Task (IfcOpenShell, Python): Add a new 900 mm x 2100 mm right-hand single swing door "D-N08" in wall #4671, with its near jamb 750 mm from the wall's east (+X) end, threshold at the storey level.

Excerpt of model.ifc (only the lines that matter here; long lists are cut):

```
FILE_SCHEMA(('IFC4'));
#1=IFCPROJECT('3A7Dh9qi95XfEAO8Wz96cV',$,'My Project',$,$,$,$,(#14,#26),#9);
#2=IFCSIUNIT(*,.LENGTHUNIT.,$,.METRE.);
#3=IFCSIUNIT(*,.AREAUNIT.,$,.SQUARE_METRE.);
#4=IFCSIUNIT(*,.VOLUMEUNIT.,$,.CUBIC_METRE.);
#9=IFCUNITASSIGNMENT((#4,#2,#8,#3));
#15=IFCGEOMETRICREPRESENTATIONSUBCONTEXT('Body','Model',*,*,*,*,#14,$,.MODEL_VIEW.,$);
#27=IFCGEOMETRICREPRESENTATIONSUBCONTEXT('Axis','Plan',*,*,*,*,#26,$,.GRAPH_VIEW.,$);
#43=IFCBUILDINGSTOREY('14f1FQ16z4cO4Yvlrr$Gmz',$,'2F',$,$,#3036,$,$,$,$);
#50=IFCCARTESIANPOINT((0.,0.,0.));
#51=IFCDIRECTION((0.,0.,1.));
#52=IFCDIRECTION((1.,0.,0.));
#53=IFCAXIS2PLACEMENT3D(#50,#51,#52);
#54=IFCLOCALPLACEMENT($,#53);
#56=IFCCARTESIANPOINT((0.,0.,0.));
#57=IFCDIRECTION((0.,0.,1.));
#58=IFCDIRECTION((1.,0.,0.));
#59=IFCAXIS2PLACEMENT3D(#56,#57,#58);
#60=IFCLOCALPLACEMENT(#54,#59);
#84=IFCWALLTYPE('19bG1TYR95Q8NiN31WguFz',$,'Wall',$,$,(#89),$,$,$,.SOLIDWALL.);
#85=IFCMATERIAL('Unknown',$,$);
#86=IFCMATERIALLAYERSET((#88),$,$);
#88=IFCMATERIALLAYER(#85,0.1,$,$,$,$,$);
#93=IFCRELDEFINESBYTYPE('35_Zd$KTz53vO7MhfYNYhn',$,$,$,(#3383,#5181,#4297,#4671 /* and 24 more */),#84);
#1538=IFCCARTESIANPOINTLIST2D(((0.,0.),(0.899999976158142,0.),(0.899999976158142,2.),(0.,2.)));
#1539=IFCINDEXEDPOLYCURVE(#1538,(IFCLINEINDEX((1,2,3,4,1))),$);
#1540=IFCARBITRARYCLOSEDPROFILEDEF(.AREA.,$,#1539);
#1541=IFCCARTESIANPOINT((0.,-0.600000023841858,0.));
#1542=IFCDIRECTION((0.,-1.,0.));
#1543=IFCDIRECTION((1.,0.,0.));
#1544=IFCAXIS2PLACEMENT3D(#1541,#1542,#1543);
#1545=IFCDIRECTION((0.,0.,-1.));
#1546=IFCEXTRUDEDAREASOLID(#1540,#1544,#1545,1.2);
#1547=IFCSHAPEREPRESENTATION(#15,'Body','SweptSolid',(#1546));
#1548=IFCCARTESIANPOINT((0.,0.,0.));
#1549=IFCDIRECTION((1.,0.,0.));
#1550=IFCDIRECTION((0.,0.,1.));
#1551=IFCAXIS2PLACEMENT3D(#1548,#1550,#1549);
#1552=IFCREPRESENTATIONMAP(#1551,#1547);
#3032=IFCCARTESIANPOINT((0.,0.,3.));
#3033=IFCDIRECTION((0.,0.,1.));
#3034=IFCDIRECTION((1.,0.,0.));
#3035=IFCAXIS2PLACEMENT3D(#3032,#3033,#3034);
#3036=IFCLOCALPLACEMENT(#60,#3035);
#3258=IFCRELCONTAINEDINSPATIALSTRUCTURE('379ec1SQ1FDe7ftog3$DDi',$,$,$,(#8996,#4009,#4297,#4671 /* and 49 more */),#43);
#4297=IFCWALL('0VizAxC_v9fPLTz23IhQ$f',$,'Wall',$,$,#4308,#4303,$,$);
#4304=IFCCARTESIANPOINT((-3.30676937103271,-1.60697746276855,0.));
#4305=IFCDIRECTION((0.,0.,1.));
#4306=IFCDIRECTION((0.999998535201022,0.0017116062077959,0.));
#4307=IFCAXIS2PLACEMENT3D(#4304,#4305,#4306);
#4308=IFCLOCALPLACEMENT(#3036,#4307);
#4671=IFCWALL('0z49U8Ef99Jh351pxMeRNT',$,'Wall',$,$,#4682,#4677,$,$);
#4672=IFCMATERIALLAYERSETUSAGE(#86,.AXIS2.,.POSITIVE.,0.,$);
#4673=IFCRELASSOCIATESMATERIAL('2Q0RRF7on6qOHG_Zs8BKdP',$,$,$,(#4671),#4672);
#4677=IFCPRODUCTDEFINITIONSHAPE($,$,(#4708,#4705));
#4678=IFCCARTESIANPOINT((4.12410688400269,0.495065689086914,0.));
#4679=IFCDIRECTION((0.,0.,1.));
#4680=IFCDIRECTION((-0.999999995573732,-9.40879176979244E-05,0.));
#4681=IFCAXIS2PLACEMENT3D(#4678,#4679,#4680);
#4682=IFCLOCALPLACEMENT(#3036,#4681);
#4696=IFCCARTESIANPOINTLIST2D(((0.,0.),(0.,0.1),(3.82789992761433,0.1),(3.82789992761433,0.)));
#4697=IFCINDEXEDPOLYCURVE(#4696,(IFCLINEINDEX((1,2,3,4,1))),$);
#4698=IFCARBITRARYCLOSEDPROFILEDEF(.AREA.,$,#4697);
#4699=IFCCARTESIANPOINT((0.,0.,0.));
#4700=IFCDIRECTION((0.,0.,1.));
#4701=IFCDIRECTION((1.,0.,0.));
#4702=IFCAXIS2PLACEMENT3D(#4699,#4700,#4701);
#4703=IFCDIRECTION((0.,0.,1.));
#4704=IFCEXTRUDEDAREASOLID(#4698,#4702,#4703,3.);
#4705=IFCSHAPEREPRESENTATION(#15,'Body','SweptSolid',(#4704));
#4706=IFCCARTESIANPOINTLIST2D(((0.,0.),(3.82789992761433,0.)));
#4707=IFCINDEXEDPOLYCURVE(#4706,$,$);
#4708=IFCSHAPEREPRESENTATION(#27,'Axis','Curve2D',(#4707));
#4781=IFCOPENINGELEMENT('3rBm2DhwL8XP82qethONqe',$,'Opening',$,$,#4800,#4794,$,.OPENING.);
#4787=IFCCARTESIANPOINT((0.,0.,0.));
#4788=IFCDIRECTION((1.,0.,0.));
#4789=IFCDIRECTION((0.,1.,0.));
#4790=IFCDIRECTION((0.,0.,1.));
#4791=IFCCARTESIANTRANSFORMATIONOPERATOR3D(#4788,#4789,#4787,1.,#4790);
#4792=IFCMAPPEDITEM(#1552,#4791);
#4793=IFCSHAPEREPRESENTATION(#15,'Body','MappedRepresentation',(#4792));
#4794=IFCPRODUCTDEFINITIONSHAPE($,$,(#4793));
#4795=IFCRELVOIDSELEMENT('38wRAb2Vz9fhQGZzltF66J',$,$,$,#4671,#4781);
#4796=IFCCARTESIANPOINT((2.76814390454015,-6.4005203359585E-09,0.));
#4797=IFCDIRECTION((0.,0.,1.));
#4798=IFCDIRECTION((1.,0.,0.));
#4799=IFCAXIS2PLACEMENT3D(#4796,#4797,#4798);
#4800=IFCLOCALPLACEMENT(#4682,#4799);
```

```python
import numpy as np
import ifcopenshell
import ifcopenshell.api.feature
import ifcopenshell.api.geometry
import ifcopenshell.api.root
import ifcopenshell.api.spatial
import ifcopenshell.geom
import ifcopenshell.util.element
import ifcopenshell.util.placement
import ifcopenshell.util.representation
import ifcopenshell.util.shape
import ifcopenshell.util.unit

model = ifcopenshell.open("model.ifc")
unit_scale = ifcopenshell.util.unit.calculate_unit_scale(model)
settings = ifcopenshell.geom.settings()


def volume(element):
    """Net volume in cubic metres, openings subtracted."""
    shape = ifcopenshell.geom.create_shape(settings, element)
    return ifcopenshell.util.shape.get_volume(shape.geometry)


wall = model.by_id(4671)
storey = ifcopenshell.util.element.get_container(wall, ifc_class="IfcBuildingStorey")
context = ifcopenshell.util.representation.get_context(model, "Model", "Body", "MODEL_VIEW")
before = volume(wall)

width, height, from_end, sill = 0.9, 2.1, 0.75, 0.0  # metres

# The wall runs along its own X axis, and the end named is its -X end.
wall_shape = ifcopenshell.geom.create_shape(settings, wall)
x, y, z = ifcopenshell.util.shape.get_vertices(wall_shape.geometry).T
start = x.min() + from_end
face, thickness = float(y.min()), float(y.max() - y.min())
wall_matrix = ifcopenshell.util.placement.get_local_placement(wall.ObjectPlacement)
level = ifcopenshell.util.placement.get_local_placement(storey.ObjectPlacement)[2, 3]


def in_wall(x, y):
    """Placement at x, y metres in the wall's axes, at sill height."""
    matrix = wall_matrix.copy()
    matrix[:, 3] = wall_matrix @ np.array([x / unit_scale, y / unit_scale, 0.0, 1.0])
    matrix[2, 3] = level + sill / unit_scale
    return matrix


# Opening: a box that overshoots both wall faces by 50 mm.
opening = ifcopenshell.api.root.create_entity(model, ifc_class="IfcOpeningElement", predefined_type="OPENING")
box = ifcopenshell.api.geometry.add_wall_representation(
    model, context=context, length=width, height=height, thickness=thickness + 0.1
)
ifcopenshell.api.geometry.assign_representation(model, product=opening, representation=box)
ifcopenshell.api.geometry.edit_object_placement(model, product=opening, matrix=in_wall(start, face - 0.05), is_si=False)
ifcopenshell.api.feature.add_feature(model, feature=opening, element=wall)

door = ifcopenshell.api.root.create_entity(model, ifc_class="IfcDoor", name="D-N08", predefined_type="DOOR")
door.OverallWidth, door.OverallHeight = width / unit_scale, height / unit_scale
door.OperationType = "SINGLE_SWING_RIGHT"
body = ifcopenshell.api.geometry.add_door_representation(
    model,
    context=context,
    overall_width=door.OverallWidth,
    overall_height=door.OverallHeight,
    operation_type="SINGLE_SWING_RIGHT",
    lining_properties={"LiningDepth": thickness / unit_scale, "ThresholdDepth": thickness / unit_scale},
)
ifcopenshell.api.geometry.assign_representation(model, product=door, representation=body)
ifcopenshell.api.spatial.assign_container(model, products=[door], relating_structure=storey)
ifcopenshell.api.feature.add_filling(model, opening=opening, element=door)

# The lining spans the wall, so the door starts at the wall face.
ifcopenshell.api.geometry.edit_object_placement(model, product=door, matrix=in_wall(start, face), is_si=False)

after = volume(wall)

print(f"wall volume {before:.3f} -> {after:.3f} m3")

model.write("model_updated.ifc")
```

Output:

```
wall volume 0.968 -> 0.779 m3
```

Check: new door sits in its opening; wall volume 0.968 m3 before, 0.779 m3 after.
